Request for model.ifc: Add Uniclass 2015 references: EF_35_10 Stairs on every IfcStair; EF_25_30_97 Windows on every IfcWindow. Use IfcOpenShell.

First a look at what the model holds.

```python
import ifcopenshell

model = ifcopenshell.open("model.ifc")
print(model.schema)
print("classifications:", [c.Name for c in model.by_type("IfcClassification")])
for ifc_class in ("IfcDoor", "IfcRoof", "IfcStair", "IfcWall", "IfcWindow"):
    print(ifc_class, len(model.by_type(ifc_class)))
```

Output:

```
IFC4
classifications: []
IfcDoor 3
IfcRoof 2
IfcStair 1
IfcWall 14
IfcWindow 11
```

```python
import ifcopenshell
import ifcopenshell.api.classification

model = ifcopenshell.open("model.ifc")

system = ifcopenshell.api.classification.add_classification(model, classification="Uniclass 2015")

codes = {
    "IfcStair": ("EF_35_10", "Stairs"),
    "IfcWindow": ("EF_25_30_97", "Windows"),
}
for ifc_class, (code, name) in codes.items():
    products = model.by_type(ifc_class)
    ifcopenshell.api.classification.add_reference(
        model, products=products, classification=system, identification=code, name=name
    )
    print(code, len(products))

model.write("model_updated.ifc")
```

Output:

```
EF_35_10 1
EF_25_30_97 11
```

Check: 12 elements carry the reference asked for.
